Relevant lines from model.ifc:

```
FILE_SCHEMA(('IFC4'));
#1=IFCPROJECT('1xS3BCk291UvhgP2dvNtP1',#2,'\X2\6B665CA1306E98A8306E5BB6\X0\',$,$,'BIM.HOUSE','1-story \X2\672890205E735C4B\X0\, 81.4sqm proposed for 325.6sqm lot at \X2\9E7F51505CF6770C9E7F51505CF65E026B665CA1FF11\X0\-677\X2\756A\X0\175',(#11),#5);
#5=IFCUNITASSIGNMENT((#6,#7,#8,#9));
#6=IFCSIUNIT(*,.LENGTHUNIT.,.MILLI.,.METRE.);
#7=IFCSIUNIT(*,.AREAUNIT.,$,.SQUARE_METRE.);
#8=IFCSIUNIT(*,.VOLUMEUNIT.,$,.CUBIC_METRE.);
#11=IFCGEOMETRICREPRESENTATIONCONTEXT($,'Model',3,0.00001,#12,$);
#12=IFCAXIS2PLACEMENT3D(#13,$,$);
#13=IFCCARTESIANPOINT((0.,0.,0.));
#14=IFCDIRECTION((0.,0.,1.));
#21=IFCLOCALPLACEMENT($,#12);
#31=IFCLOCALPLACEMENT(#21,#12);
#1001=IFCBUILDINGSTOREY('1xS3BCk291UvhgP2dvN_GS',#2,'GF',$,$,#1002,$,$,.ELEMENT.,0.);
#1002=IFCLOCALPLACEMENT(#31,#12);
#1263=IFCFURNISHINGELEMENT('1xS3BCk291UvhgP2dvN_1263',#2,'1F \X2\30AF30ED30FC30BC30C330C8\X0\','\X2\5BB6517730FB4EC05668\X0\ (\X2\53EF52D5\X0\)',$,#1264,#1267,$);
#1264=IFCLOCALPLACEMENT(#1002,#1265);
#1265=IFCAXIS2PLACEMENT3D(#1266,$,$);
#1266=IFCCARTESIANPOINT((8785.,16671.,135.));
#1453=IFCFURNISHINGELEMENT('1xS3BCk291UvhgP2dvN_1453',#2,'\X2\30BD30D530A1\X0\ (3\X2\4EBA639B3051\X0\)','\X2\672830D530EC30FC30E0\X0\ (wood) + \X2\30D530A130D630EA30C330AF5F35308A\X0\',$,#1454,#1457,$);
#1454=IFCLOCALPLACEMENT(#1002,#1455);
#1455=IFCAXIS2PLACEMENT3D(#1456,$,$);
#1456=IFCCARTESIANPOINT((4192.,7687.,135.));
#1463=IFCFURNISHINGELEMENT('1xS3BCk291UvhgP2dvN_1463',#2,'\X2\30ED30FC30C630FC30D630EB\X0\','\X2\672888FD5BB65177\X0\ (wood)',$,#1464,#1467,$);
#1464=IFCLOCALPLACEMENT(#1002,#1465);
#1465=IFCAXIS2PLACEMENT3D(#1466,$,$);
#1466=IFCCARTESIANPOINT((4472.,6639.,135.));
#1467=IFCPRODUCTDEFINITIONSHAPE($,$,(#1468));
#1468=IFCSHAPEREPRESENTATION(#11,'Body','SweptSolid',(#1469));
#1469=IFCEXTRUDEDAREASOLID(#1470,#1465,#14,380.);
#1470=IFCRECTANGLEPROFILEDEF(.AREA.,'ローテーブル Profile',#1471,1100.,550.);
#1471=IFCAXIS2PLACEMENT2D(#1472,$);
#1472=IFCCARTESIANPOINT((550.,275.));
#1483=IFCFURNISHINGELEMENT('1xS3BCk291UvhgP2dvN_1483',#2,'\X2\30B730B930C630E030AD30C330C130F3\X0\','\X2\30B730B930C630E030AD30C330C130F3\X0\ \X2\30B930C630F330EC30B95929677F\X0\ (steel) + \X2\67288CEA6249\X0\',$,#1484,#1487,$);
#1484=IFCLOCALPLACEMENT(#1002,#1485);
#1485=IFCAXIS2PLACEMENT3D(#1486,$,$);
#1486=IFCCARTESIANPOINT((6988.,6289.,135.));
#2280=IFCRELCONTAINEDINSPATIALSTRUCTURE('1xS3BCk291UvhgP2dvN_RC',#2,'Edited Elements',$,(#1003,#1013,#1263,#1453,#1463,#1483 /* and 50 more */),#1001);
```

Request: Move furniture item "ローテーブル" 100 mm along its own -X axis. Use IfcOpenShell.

```python
import ifcopenshell
import ifcopenshell.api.geometry
import ifcopenshell.util.placement
import ifcopenshell.util.unit

model = ifcopenshell.open("model.ifc")
unit_scale = ifcopenshell.util.unit.calculate_unit_scale(model)

item = model.by_guid("1xS3BCk291UvhgP2dvN_1463")
matrix = ifcopenshell.util.placement.get_local_placement(item.ObjectPlacement)
matrix[:3, 3] -= matrix[:3, 0] * 0.1 / unit_scale
ifcopenshell.api.geometry.edit_object_placement(model, product=item, matrix=matrix, is_si=False)

print(ifcopenshell.util.placement.get_local_placement(item.ObjectPlacement).round(3) + 0.0)

model.write("model_edited.ifc")
```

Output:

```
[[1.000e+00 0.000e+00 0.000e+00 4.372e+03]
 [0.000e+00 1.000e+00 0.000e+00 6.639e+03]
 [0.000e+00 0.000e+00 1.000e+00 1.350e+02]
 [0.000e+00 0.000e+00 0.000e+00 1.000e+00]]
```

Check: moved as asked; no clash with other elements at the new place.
